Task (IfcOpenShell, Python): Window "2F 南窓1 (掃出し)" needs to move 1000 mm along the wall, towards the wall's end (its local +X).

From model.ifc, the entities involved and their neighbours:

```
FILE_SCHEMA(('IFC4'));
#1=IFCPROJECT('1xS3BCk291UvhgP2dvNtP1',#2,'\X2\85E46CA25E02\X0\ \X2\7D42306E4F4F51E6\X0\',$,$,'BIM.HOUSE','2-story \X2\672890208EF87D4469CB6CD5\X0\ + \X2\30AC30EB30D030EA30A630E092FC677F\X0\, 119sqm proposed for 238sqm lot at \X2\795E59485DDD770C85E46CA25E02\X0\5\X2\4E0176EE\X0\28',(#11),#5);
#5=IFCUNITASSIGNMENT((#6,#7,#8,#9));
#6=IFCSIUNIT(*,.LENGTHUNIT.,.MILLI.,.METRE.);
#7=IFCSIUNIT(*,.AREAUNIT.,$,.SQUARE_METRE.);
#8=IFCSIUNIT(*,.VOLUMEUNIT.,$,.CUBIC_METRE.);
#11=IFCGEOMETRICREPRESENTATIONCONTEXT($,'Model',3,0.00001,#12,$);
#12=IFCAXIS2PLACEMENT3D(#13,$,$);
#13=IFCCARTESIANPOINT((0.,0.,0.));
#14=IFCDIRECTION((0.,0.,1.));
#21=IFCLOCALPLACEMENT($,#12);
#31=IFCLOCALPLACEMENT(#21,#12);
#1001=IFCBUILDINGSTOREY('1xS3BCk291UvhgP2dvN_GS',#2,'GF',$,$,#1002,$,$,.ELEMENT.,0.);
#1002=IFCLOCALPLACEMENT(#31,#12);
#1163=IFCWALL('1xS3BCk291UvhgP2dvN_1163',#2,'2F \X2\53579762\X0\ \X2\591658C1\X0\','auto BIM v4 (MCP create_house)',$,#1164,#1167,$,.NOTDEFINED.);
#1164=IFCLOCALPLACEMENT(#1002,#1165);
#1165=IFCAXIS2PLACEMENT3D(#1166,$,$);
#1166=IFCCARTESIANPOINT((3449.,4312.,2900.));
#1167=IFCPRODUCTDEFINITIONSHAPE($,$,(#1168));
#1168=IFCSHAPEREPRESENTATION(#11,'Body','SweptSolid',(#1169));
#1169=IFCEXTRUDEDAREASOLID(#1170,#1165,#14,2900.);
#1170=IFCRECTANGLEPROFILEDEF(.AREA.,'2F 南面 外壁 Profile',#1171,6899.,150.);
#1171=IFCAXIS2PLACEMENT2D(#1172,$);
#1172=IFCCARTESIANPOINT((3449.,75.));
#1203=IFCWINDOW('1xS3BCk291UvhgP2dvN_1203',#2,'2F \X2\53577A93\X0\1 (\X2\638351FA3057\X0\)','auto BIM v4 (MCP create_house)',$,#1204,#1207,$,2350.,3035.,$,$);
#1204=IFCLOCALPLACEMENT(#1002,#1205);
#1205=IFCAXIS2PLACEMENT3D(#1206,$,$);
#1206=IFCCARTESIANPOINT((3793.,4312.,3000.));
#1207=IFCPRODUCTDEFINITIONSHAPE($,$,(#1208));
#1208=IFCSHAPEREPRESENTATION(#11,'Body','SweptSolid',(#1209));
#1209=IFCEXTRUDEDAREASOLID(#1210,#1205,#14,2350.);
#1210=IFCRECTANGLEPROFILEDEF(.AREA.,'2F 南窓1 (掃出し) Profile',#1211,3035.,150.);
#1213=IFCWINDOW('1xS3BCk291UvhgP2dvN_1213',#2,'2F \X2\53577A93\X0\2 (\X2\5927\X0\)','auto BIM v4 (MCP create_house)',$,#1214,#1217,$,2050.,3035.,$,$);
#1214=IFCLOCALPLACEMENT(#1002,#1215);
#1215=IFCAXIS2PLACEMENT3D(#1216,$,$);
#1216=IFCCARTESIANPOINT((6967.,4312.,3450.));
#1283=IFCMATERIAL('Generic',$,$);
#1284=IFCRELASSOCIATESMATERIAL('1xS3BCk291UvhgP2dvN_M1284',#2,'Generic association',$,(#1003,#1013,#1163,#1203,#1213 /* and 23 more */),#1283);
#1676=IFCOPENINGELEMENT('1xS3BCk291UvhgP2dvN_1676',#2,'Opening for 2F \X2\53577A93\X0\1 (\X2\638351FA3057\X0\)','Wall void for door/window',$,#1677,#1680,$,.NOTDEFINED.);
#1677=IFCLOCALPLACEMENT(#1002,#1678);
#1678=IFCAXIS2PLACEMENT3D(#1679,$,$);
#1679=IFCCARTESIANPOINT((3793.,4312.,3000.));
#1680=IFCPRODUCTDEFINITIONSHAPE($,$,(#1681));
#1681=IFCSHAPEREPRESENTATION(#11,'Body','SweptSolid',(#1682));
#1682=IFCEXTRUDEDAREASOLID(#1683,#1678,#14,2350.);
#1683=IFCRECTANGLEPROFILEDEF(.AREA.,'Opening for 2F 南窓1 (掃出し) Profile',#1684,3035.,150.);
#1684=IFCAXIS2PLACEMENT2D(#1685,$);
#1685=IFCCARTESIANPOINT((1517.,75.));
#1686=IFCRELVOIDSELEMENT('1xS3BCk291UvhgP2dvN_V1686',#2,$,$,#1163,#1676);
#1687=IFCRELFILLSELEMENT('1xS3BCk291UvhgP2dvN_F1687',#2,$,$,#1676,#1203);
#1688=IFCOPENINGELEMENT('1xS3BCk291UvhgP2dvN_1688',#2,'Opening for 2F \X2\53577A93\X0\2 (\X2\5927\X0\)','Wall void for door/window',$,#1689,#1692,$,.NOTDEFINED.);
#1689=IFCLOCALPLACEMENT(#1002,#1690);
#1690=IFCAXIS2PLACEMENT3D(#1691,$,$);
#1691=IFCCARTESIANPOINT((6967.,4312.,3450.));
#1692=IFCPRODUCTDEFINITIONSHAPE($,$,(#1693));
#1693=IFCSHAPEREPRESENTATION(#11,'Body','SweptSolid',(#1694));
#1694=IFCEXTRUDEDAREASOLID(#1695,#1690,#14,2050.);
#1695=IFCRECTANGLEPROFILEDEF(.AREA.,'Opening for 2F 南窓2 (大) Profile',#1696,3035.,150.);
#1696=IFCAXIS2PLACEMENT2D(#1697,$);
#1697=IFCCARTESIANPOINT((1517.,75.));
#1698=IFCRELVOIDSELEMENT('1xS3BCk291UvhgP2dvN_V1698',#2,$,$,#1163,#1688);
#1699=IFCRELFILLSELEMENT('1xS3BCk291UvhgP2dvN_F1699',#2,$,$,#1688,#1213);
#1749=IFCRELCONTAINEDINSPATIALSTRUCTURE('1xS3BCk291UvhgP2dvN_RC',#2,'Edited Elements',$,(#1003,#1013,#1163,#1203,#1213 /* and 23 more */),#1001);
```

```python
import ifcopenshell
import ifcopenshell.api.geometry
import ifcopenshell.util.placement

model = ifcopenshell.open("model.ifc")

window = model.by_guid("1xS3BCk291UvhgP2dvN_1203")
opening = window.FillsVoids[0].RelatingOpeningElement
wall = opening.VoidsElements[0].RelatingBuildingElement

wall_matrix = ifcopenshell.util.placement.get_local_placement(wall.ObjectPlacement)
shift = wall_matrix[:3, 0] * 1000.0
before = ifcopenshell.util.placement.get_local_placement(window.ObjectPlacement)[:3, 3].copy()

# The window is not placed relative to its opening, so move both.
for product in (opening, window):
    matrix = ifcopenshell.util.placement.get_local_placement(product.ObjectPlacement)
    matrix[:3, 3] += shift
    ifcopenshell.api.geometry.edit_object_placement(model, product=product, matrix=matrix, is_si=False)

after = ifcopenshell.util.placement.get_local_placement(window.ObjectPlacement)[:3, 3]
print("window moved by", (after - before).round(3) + 0.0)

model.write("model-out.ifc")
```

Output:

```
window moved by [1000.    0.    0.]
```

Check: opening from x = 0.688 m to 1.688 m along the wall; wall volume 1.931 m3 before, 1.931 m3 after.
